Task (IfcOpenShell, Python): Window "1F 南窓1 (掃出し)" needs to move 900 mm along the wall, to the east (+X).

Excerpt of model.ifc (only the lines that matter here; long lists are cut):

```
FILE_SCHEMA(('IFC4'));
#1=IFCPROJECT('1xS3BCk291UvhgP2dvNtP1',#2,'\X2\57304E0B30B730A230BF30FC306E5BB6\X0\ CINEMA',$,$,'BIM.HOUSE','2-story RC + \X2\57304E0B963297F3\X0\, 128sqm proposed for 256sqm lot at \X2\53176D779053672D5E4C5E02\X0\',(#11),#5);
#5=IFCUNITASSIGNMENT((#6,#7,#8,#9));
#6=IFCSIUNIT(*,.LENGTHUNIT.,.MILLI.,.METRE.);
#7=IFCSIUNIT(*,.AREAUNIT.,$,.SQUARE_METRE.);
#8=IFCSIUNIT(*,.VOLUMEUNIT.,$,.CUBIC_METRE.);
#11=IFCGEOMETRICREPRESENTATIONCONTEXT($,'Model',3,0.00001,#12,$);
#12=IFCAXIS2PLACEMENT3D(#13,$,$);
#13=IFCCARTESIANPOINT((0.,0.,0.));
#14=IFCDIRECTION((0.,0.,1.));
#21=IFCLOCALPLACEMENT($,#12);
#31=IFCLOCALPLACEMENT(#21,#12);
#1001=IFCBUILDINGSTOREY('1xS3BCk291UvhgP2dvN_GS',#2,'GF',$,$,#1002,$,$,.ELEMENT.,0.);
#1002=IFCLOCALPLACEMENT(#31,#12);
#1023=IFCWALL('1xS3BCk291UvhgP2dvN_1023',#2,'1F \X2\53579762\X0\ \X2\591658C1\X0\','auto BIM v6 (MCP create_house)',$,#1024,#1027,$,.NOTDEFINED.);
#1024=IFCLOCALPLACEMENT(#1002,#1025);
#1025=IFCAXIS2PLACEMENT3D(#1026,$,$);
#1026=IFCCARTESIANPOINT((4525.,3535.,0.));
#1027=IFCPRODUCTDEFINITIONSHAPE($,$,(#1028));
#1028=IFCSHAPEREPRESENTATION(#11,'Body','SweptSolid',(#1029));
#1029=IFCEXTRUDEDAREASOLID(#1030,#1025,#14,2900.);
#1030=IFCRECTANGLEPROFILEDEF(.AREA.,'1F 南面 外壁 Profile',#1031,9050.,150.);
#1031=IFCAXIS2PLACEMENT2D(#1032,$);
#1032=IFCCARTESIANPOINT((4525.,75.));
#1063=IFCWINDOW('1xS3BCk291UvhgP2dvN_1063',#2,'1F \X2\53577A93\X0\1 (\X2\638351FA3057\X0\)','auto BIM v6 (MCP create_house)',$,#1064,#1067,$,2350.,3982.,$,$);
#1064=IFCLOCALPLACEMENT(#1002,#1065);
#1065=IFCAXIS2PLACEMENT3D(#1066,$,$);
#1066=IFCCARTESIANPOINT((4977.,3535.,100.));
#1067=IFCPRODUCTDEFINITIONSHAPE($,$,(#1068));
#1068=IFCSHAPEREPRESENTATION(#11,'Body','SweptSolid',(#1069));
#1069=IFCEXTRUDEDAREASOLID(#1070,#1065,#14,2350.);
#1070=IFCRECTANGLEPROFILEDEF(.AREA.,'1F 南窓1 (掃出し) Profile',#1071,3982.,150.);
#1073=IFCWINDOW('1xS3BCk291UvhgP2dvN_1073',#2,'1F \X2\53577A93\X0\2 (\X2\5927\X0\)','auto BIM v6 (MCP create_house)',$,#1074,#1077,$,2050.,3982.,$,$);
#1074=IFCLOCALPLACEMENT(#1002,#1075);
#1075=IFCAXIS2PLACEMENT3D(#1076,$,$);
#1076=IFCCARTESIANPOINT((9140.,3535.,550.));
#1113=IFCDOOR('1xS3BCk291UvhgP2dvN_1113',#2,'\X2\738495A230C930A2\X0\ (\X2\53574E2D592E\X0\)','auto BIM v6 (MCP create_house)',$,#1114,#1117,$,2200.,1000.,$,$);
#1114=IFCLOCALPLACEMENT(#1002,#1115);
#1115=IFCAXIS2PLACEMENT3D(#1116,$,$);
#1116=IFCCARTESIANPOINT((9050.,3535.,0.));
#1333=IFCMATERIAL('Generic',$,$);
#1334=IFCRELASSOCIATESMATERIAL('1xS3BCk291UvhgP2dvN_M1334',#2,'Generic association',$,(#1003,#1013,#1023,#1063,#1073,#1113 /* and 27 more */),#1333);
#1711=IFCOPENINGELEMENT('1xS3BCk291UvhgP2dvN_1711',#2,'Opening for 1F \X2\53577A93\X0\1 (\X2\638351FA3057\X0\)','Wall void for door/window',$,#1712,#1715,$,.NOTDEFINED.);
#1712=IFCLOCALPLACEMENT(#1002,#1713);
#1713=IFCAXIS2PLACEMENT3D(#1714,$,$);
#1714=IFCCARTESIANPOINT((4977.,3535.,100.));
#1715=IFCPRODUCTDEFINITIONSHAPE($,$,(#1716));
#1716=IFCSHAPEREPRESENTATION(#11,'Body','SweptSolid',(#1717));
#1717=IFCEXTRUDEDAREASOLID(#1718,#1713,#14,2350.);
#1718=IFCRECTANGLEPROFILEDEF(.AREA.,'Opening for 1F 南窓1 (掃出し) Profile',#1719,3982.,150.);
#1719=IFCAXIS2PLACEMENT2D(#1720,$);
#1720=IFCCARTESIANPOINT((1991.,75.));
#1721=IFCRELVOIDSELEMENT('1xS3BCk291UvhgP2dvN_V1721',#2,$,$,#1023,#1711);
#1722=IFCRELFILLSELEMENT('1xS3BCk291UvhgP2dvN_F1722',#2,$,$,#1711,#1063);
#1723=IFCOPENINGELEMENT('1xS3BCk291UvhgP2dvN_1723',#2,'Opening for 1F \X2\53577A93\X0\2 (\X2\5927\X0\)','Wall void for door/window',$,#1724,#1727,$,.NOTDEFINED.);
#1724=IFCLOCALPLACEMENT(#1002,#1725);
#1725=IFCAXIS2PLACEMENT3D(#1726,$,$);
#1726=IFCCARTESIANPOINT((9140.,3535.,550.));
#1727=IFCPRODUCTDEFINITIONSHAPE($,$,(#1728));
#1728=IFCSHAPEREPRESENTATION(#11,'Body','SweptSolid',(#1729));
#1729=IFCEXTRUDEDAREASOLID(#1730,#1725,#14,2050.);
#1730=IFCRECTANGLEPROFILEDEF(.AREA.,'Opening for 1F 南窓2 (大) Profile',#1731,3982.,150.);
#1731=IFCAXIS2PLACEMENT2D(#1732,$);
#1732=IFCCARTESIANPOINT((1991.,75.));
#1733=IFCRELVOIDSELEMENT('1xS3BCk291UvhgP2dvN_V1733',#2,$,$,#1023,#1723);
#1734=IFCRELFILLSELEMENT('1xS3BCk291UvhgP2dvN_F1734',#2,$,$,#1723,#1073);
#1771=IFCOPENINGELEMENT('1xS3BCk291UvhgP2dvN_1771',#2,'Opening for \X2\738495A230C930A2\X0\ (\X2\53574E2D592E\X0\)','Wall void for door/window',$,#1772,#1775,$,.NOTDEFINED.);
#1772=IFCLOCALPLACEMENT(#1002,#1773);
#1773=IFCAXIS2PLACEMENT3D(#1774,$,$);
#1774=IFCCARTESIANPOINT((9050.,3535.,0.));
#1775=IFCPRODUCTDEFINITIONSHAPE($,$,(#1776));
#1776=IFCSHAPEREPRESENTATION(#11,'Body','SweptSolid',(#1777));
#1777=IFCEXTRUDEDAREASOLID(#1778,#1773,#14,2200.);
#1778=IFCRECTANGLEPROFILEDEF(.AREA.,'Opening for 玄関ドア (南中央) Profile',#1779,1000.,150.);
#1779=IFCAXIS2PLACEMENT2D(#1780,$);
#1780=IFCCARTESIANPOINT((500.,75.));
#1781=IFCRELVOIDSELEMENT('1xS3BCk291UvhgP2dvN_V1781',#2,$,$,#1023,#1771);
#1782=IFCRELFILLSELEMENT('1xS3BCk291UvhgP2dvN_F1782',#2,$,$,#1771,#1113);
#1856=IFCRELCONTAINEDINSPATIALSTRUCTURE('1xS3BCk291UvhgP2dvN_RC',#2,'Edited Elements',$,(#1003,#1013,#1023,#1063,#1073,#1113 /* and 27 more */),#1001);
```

```python
import ifcopenshell
import ifcopenshell.api.geometry
import ifcopenshell.util.placement
import ifcopenshell.util.unit

model = ifcopenshell.open("model.ifc")
unit_scale = ifcopenshell.util.unit.calculate_unit_scale(model)

window = model.by_guid("1xS3BCk291UvhgP2dvN_1063")
opening = window.FillsVoids[0].RelatingOpeningElement
wall = opening.VoidsElements[0].RelatingBuildingElement

wall_matrix = ifcopenshell.util.placement.get_local_placement(wall.ObjectPlacement)
shift = wall_matrix[:3, 0] * 0.9 / unit_scale
before = ifcopenshell.util.placement.get_local_placement(window.ObjectPlacement)[:3, 3].copy()

# The window is not placed relative to its opening, so move both.
for product in (opening, window):
    matrix = ifcopenshell.util.placement.get_local_placement(product.ObjectPlacement)
    matrix[:3, 3] += shift
    ifcopenshell.api.geometry.edit_object_placement(model, product=product, matrix=matrix, is_si=False)

after = ifcopenshell.util.placement.get_local_placement(window.ObjectPlacement)[:3, 3]
print("window moved by", (after - before).round(3) + 0.0)

model.write("model_v2.ifc")
```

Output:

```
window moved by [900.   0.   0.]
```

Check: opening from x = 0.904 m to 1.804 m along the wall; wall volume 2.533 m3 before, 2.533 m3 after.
